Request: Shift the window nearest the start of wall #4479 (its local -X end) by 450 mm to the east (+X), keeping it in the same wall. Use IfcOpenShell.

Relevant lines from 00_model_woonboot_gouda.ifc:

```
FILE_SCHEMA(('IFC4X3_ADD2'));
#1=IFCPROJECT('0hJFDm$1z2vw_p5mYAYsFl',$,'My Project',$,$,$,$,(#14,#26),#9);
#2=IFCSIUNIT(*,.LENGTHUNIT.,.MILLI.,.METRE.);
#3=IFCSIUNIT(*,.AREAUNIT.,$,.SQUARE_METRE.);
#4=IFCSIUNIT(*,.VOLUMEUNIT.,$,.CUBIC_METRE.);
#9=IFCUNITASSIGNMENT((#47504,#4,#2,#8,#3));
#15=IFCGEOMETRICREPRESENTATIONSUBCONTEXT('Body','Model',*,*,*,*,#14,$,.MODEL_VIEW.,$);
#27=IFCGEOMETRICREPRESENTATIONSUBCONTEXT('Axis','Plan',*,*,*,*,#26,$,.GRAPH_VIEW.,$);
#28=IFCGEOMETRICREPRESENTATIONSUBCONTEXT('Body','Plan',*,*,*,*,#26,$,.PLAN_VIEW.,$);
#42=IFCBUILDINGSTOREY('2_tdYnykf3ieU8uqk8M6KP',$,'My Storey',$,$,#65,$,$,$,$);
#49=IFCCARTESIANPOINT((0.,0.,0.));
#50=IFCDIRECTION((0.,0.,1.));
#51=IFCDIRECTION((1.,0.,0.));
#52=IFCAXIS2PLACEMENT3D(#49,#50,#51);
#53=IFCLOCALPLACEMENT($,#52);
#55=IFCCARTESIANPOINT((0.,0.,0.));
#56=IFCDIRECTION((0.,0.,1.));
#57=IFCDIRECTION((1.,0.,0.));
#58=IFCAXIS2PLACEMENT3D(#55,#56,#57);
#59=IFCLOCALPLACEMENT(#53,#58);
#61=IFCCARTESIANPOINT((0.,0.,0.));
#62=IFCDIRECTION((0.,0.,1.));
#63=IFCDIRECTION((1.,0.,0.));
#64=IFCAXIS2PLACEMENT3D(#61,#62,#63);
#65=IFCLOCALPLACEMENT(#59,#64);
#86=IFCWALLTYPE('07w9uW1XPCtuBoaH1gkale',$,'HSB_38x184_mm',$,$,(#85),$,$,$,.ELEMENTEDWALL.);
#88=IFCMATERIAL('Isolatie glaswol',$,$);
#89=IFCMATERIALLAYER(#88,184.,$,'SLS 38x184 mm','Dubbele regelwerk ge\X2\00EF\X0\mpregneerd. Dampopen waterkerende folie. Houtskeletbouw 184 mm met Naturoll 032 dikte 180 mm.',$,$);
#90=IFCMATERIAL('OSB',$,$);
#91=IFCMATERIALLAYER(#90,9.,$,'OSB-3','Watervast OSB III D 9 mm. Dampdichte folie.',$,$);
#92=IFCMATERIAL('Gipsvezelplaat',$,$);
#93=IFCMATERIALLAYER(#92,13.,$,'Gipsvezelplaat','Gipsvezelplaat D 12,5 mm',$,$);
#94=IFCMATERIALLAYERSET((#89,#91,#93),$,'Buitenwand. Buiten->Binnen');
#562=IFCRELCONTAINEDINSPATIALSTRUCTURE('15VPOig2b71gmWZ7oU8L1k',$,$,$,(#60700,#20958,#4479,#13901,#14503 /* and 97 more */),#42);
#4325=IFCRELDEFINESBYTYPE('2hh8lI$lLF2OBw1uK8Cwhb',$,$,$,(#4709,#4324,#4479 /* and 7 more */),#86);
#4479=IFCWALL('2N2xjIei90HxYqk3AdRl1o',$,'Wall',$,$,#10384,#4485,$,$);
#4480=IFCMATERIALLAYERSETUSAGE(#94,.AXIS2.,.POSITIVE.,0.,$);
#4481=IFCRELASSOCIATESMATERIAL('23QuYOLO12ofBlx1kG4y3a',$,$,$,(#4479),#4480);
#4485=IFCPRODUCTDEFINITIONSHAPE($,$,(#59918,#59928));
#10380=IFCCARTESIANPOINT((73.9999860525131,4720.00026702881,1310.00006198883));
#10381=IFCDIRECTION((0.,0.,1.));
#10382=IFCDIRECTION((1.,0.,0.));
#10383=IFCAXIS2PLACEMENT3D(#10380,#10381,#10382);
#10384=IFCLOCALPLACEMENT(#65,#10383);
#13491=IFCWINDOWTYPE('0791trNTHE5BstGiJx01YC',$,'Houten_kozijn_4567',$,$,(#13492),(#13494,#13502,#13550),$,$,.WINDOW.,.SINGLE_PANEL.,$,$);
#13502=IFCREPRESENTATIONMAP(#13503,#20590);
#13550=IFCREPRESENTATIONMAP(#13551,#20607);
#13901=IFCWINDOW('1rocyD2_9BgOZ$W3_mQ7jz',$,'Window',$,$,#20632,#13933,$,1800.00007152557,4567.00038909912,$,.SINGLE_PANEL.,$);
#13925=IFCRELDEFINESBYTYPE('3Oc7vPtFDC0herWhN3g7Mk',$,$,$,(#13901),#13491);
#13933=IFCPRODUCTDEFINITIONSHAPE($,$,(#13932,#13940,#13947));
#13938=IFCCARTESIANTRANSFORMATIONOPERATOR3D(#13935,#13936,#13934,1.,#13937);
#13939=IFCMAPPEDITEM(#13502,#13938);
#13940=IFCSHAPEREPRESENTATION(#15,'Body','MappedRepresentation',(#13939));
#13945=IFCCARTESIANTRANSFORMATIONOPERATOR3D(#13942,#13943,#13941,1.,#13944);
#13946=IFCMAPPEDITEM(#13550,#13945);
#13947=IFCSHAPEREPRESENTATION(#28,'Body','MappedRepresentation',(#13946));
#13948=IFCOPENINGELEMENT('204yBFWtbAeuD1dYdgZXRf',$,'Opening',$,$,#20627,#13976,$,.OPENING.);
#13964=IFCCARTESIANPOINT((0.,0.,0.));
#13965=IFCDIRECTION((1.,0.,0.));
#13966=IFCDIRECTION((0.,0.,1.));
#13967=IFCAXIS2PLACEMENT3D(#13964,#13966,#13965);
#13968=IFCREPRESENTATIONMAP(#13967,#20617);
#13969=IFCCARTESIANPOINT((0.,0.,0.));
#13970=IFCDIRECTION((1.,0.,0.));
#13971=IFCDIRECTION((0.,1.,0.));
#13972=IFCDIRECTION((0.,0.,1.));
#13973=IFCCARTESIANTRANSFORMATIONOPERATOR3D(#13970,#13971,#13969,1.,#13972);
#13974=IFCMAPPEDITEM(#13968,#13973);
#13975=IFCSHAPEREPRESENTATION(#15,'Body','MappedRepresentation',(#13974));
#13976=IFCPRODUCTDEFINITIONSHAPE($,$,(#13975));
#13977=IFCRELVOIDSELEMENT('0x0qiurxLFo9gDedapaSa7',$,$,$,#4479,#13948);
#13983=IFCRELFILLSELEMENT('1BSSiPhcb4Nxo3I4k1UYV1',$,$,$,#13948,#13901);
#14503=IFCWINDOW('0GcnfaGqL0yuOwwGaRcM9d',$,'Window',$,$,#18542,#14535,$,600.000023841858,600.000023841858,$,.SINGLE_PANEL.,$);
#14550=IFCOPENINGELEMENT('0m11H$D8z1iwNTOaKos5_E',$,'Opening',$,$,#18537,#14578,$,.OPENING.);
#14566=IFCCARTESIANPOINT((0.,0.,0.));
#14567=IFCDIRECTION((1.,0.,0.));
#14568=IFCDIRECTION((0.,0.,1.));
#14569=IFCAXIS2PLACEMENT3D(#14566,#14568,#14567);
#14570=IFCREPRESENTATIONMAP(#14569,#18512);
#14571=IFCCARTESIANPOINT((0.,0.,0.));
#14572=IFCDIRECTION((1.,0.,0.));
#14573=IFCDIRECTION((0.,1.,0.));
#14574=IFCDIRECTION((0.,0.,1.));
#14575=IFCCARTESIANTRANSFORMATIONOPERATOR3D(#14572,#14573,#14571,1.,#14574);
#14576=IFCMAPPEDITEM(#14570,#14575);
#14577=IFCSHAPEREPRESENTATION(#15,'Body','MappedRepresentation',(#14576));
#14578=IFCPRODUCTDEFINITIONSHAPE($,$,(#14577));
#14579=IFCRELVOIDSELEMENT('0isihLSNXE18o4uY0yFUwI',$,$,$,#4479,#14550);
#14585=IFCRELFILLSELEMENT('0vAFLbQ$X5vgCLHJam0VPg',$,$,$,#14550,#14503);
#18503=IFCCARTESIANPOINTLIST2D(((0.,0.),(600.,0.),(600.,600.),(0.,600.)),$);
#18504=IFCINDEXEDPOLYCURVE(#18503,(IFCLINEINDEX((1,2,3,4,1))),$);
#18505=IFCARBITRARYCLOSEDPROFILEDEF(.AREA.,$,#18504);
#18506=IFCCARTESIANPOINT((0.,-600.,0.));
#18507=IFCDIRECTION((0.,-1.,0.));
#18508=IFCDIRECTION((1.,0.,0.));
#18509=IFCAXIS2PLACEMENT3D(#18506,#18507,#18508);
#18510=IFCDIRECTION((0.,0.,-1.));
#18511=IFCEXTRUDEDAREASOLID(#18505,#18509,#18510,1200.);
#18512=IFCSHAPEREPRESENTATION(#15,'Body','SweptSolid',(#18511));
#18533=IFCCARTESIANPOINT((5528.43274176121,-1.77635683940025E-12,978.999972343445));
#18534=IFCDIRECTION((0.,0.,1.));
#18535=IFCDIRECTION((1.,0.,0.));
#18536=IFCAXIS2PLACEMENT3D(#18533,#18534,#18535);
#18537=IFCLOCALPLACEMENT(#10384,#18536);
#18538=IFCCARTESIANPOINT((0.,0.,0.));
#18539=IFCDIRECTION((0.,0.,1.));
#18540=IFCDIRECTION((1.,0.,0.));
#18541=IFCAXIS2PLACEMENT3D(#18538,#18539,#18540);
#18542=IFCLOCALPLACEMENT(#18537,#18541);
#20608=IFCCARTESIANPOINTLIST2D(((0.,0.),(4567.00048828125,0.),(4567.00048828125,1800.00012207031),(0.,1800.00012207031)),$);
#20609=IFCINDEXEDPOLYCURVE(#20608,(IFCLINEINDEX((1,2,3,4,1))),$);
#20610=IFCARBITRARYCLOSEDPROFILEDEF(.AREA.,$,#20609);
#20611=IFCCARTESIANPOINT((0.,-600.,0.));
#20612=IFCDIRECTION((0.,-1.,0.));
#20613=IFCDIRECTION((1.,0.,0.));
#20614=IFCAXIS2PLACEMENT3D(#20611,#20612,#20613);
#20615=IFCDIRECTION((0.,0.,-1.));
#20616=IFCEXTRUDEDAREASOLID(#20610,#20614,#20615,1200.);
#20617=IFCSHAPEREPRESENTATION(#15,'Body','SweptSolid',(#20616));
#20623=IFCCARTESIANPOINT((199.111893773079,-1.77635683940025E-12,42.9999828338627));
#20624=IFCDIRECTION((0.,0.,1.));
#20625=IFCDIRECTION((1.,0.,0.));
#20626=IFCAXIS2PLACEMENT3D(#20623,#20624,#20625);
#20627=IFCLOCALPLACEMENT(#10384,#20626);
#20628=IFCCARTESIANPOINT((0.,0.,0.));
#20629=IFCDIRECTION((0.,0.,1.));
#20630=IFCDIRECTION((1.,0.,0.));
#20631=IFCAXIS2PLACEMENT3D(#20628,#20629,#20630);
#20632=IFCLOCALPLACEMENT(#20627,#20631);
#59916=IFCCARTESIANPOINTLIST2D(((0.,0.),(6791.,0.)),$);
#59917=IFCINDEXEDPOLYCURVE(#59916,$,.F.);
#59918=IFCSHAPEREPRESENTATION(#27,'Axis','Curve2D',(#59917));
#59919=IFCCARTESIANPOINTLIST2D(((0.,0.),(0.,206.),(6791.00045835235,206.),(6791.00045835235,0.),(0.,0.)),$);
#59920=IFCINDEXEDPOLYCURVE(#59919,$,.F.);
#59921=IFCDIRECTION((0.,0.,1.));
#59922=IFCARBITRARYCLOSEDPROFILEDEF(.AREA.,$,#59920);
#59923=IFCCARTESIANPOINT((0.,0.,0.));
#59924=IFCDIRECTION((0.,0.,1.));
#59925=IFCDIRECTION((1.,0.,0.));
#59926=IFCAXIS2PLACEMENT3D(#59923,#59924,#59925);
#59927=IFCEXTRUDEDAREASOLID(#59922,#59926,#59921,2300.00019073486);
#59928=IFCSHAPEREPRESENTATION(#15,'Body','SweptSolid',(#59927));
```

```python
import ifcopenshell
import ifcopenshell.api.geometry
import ifcopenshell.util.placement
import ifcopenshell.util.unit

model = ifcopenshell.open("00_model_woonboot_gouda.ifc")
unit_scale = ifcopenshell.util.unit.calculate_unit_scale(model)

window = model.by_guid("1rocyD2_9BgOZ$W3_mQ7jz")
opening = window.FillsVoids[0].RelatingOpeningElement
wall = opening.VoidsElements[0].RelatingBuildingElement

wall_matrix = ifcopenshell.util.placement.get_local_placement(wall.ObjectPlacement)
shift = wall_matrix[:3, 0] * 0.45 / unit_scale
before = ifcopenshell.util.placement.get_local_placement(window.ObjectPlacement)[:3, 3].copy()

# The window is placed relative to its opening, so it follows when the opening moves.
matrix = ifcopenshell.util.placement.get_local_placement(opening.ObjectPlacement)
matrix[:3, 3] += shift
ifcopenshell.api.geometry.edit_object_placement(
    model, product=opening, matrix=matrix, is_si=False, should_transform_children=True
)

after = ifcopenshell.util.placement.get_local_placement(window.ObjectPlacement)[:3, 3]
print("window moved by", (after - before).round(3) + 0.0)

model.write("00_model_woonboot_gouda_updated.ifc")
```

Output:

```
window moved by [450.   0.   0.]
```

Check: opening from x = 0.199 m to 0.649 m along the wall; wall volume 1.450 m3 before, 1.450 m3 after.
